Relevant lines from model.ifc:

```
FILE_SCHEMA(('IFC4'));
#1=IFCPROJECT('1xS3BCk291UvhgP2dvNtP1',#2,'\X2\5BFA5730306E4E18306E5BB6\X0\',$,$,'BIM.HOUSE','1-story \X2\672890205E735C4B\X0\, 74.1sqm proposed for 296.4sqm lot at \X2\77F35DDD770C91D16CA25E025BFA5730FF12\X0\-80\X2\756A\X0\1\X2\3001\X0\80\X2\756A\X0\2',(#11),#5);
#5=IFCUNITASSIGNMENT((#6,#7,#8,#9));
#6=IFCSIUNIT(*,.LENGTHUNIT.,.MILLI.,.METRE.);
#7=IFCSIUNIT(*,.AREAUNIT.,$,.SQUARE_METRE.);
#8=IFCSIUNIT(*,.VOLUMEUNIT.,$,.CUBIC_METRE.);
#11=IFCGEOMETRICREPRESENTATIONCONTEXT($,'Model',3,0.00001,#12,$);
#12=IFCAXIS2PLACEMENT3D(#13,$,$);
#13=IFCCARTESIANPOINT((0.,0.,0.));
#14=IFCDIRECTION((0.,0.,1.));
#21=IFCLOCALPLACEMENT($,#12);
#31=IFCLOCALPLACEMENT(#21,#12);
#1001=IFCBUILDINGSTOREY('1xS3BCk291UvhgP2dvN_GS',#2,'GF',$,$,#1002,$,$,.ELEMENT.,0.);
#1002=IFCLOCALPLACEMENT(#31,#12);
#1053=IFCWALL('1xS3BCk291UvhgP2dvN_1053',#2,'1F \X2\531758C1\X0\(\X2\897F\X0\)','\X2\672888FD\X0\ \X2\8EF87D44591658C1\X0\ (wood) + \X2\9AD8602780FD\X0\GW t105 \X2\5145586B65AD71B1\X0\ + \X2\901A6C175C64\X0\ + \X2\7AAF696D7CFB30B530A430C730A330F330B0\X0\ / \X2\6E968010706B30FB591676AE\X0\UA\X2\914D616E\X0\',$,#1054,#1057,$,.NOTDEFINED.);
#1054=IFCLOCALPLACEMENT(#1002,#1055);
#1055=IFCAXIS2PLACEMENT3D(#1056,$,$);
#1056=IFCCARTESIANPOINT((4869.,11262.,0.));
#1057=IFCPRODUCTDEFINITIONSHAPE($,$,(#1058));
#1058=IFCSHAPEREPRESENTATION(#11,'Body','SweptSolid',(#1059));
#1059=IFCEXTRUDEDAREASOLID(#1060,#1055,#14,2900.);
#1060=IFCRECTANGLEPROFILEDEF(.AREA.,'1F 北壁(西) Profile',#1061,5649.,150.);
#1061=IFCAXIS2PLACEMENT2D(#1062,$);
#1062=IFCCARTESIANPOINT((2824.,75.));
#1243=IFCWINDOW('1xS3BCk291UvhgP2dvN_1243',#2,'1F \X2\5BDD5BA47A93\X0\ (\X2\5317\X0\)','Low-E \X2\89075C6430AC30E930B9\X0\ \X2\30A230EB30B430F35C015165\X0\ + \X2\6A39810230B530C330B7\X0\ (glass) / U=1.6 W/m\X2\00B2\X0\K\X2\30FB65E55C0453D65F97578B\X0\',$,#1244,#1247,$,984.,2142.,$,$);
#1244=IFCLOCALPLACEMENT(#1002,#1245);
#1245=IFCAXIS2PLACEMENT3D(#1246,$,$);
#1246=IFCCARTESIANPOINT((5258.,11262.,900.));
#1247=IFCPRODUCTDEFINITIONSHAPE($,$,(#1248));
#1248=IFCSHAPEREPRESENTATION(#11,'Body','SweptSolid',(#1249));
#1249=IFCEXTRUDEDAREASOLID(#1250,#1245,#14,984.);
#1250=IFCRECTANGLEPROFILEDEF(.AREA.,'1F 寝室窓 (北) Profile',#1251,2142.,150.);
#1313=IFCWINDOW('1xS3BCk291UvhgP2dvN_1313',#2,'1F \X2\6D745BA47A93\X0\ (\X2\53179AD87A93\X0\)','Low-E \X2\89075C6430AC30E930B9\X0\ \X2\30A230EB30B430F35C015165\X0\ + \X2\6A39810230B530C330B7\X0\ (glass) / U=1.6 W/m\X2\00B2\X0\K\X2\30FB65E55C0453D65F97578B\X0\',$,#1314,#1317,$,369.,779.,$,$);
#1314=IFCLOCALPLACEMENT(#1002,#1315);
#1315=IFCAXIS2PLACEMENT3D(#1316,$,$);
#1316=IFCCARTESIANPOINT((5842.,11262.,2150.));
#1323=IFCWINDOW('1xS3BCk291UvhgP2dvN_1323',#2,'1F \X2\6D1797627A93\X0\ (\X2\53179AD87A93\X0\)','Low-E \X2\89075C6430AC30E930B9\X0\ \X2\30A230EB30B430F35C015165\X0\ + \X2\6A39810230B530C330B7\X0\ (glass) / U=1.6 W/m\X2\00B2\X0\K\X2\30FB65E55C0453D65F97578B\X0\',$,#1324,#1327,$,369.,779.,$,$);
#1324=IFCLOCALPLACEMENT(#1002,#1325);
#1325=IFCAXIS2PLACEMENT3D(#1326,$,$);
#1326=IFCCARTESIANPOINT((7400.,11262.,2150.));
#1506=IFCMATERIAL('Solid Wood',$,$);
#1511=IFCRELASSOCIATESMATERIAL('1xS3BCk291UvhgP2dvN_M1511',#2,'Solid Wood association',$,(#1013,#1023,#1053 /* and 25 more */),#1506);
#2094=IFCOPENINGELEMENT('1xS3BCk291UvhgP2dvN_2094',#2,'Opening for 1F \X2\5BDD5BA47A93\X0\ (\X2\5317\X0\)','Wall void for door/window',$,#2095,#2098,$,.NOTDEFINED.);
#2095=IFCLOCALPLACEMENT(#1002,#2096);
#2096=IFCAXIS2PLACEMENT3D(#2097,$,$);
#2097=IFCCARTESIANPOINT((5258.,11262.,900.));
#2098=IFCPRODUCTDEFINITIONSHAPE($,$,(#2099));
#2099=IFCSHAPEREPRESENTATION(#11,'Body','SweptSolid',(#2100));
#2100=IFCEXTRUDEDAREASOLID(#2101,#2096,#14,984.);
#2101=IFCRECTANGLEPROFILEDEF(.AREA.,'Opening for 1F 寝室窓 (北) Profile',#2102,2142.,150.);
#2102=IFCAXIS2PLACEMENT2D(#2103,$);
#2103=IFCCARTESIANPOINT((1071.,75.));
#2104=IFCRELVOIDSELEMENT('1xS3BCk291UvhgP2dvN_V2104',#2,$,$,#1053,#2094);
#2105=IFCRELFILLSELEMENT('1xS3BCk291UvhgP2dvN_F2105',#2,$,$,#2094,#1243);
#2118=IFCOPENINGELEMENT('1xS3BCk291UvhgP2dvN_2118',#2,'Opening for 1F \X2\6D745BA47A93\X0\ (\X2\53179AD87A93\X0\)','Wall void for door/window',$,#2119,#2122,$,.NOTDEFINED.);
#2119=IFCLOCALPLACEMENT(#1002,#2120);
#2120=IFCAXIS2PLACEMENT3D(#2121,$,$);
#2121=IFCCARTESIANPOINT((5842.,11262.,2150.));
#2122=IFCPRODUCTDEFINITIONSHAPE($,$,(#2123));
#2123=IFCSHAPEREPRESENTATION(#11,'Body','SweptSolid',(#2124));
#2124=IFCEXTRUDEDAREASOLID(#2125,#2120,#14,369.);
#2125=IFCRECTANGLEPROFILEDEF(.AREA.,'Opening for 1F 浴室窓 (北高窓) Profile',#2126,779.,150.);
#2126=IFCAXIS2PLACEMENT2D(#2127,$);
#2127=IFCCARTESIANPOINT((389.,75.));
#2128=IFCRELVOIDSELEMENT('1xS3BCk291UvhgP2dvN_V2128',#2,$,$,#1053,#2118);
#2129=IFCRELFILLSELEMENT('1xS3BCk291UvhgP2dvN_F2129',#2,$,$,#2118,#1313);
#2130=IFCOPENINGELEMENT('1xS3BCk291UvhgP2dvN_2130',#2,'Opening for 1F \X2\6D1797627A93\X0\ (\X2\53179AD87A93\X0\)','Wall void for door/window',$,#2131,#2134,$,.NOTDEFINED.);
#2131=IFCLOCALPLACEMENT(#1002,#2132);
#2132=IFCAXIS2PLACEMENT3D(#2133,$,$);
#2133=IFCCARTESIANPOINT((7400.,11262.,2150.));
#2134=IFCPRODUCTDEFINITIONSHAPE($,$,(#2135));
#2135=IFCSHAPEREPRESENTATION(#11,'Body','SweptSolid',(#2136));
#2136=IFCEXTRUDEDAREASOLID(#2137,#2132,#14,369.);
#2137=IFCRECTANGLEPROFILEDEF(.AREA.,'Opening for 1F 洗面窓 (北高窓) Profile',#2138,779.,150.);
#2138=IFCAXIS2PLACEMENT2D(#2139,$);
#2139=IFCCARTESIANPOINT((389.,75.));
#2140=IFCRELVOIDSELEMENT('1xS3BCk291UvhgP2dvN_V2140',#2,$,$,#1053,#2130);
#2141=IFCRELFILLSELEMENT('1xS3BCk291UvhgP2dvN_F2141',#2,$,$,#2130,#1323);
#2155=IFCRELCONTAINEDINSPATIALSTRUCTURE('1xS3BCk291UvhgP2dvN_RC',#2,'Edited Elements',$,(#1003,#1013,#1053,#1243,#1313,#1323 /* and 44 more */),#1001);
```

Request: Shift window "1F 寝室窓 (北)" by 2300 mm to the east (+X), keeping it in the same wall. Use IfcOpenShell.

```python
import ifcopenshell
import ifcopenshell.api.geometry
import ifcopenshell.util.placement

model = ifcopenshell.open("model.ifc")

window = model.by_guid("1xS3BCk291UvhgP2dvN_1243")
opening = window.FillsVoids[0].RelatingOpeningElement
wall = opening.VoidsElements[0].RelatingBuildingElement

wall_matrix = ifcopenshell.util.placement.get_local_placement(wall.ObjectPlacement)
shift = wall_matrix[:3, 0] * 2300.0
before = ifcopenshell.util.placement.get_local_placement(window.ObjectPlacement)[:3, 3].copy()

# The window is not placed relative to its opening, so move both.
for product in (opening, window):
    matrix = ifcopenshell.util.placement.get_local_placement(product.ObjectPlacement)
    matrix[:3, 3] += shift
    ifcopenshell.api.geometry.edit_object_placement(model, product=product, matrix=matrix, is_si=False)

after = ifcopenshell.util.placement.get_local_placement(window.ObjectPlacement)[:3, 3]
print("window moved by", (after - before).round(3) + 0.0)

model.write("model_updated.ifc")
```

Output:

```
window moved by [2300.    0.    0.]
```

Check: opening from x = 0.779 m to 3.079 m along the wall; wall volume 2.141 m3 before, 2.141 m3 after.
